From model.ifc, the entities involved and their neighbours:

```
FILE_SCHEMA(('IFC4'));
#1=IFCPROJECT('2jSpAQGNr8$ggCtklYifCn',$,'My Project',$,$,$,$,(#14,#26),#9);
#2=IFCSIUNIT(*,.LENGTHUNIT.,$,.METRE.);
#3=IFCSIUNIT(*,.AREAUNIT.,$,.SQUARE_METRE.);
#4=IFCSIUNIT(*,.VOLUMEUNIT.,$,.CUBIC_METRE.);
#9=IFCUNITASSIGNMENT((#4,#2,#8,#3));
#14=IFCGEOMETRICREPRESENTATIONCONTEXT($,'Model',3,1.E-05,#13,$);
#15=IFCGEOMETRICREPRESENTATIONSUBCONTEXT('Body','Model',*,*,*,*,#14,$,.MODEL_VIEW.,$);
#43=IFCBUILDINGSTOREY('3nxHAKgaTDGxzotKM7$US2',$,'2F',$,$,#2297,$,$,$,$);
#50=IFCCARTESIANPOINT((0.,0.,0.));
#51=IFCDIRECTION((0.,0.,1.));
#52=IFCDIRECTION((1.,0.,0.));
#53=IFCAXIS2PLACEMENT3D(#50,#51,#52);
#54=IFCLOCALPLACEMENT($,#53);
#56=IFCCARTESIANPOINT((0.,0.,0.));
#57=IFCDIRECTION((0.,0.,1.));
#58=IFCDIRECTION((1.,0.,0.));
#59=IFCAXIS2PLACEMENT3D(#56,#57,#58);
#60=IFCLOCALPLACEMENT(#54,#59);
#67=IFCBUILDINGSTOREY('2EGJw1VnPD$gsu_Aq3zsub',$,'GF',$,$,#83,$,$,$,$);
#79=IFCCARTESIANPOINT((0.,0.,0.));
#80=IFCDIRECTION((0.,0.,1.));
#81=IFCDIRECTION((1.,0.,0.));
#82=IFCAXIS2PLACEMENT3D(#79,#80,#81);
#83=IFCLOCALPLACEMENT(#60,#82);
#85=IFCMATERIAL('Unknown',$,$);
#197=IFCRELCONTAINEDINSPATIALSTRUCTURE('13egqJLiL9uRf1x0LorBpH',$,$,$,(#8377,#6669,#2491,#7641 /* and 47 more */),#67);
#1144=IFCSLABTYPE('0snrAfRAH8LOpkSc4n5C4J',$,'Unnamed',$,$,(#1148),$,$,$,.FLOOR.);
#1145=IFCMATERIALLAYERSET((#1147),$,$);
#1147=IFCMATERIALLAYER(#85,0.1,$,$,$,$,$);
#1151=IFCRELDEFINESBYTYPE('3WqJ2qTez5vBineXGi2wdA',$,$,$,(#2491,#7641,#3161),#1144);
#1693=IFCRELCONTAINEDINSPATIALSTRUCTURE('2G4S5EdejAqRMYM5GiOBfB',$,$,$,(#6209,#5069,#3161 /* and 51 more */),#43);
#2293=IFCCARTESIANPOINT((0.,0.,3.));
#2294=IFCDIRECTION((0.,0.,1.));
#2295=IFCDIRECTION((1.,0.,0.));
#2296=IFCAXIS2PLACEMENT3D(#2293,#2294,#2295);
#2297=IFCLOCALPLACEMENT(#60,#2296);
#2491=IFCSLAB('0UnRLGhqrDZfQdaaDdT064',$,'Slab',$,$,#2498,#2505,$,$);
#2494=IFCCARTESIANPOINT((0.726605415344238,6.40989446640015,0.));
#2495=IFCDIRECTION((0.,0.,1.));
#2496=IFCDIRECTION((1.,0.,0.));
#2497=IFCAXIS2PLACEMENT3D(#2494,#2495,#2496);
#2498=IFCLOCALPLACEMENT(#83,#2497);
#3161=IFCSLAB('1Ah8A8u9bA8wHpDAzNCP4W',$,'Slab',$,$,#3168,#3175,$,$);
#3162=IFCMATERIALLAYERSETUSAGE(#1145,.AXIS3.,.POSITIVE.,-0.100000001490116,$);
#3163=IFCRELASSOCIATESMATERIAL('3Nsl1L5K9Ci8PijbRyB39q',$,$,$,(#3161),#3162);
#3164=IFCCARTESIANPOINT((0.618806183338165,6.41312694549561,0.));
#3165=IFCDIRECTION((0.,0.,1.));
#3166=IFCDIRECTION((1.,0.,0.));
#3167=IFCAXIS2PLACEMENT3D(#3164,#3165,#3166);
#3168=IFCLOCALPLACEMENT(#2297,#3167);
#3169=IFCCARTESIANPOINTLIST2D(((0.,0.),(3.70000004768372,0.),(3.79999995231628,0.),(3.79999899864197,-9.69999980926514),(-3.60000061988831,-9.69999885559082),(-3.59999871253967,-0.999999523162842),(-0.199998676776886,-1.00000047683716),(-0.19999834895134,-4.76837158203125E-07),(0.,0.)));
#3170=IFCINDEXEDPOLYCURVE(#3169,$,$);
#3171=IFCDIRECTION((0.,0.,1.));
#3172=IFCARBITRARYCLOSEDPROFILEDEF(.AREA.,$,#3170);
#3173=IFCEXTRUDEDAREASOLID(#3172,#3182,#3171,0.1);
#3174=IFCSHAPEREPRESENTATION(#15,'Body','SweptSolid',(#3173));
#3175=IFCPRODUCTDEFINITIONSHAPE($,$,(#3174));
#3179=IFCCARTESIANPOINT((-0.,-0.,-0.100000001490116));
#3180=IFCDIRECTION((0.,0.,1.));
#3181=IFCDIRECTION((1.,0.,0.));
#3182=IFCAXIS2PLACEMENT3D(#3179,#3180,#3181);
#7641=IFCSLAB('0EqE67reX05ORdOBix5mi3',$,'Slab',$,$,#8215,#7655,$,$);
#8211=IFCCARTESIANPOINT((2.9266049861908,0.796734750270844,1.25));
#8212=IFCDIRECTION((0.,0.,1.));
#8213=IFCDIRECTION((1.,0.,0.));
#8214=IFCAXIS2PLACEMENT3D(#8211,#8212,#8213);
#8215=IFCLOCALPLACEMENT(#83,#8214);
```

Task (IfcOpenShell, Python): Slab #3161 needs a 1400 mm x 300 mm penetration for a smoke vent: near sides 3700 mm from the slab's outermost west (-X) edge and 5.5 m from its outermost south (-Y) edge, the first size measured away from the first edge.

```python
import numpy as np
import ifcopenshell
import ifcopenshell.api.feature
import ifcopenshell.api.geometry
import ifcopenshell.api.root
import ifcopenshell.geom
import ifcopenshell.util.placement
import ifcopenshell.util.representation
import ifcopenshell.util.shape
import ifcopenshell.util.unit

model = ifcopenshell.open("model.ifc")
unit_scale = ifcopenshell.util.unit.calculate_unit_scale(model)
settings = ifcopenshell.geom.settings()


def volume(element):
    """Net volume in cubic metres, openings subtracted."""
    shape = ifcopenshell.geom.create_shape(settings, element)
    return ifcopenshell.util.shape.get_volume(shape.geometry)


slab = model.by_guid("1Ah8A8u9bA8wHpDAzNCP4W")
before = volume(slab)

# Extent in the slab's own axes, in metres. The edges named are its -X and -Y sides.
slab_shape = ifcopenshell.geom.create_shape(settings, slab)
vertices = ifcopenshell.util.shape.get_vertices(slab_shape.geometry)
x_min, y_min, bottom = vertices.min(axis=0)
top = vertices[:, 2].max()

opening = ifcopenshell.api.root.create_entity(model, ifc_class="IfcOpeningElement", name="Smoke vent opening", predefined_type="OPENING")
context = ifcopenshell.util.representation.get_context(model, "Model", "Body", "MODEL_VIEW")
width, depth = 1.4, 0.3
outline = [(0.0, 0.0), (width, 0.0), (width, depth), (0.0, depth), (0.0, 0.0)]
# Overshoot both faces by 50 mm so the cut is clean.
shape = ifcopenshell.api.geometry.add_slab_representation(
    model, context=context, depth=top - bottom + 0.1, polyline=outline
)
ifcopenshell.api.geometry.assign_representation(model, product=opening, representation=shape)

matrix = ifcopenshell.util.placement.get_local_placement(slab.ObjectPlacement)
matrix[:, 3] = matrix @ np.append(np.array([x_min + 3.7, y_min + 5.5, bottom - 0.05]) / unit_scale, 1.0)
ifcopenshell.api.geometry.edit_object_placement(model, product=opening, matrix=matrix, is_si=False)
ifcopenshell.api.feature.add_feature(model, feature=opening, element=slab)

after = volume(slab)

print(f"slab volume {before:.3f} -> {after:.3f} m3")

model.write("model-out.ifc")
```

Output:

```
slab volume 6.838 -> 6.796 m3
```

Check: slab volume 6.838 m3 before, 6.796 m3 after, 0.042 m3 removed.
